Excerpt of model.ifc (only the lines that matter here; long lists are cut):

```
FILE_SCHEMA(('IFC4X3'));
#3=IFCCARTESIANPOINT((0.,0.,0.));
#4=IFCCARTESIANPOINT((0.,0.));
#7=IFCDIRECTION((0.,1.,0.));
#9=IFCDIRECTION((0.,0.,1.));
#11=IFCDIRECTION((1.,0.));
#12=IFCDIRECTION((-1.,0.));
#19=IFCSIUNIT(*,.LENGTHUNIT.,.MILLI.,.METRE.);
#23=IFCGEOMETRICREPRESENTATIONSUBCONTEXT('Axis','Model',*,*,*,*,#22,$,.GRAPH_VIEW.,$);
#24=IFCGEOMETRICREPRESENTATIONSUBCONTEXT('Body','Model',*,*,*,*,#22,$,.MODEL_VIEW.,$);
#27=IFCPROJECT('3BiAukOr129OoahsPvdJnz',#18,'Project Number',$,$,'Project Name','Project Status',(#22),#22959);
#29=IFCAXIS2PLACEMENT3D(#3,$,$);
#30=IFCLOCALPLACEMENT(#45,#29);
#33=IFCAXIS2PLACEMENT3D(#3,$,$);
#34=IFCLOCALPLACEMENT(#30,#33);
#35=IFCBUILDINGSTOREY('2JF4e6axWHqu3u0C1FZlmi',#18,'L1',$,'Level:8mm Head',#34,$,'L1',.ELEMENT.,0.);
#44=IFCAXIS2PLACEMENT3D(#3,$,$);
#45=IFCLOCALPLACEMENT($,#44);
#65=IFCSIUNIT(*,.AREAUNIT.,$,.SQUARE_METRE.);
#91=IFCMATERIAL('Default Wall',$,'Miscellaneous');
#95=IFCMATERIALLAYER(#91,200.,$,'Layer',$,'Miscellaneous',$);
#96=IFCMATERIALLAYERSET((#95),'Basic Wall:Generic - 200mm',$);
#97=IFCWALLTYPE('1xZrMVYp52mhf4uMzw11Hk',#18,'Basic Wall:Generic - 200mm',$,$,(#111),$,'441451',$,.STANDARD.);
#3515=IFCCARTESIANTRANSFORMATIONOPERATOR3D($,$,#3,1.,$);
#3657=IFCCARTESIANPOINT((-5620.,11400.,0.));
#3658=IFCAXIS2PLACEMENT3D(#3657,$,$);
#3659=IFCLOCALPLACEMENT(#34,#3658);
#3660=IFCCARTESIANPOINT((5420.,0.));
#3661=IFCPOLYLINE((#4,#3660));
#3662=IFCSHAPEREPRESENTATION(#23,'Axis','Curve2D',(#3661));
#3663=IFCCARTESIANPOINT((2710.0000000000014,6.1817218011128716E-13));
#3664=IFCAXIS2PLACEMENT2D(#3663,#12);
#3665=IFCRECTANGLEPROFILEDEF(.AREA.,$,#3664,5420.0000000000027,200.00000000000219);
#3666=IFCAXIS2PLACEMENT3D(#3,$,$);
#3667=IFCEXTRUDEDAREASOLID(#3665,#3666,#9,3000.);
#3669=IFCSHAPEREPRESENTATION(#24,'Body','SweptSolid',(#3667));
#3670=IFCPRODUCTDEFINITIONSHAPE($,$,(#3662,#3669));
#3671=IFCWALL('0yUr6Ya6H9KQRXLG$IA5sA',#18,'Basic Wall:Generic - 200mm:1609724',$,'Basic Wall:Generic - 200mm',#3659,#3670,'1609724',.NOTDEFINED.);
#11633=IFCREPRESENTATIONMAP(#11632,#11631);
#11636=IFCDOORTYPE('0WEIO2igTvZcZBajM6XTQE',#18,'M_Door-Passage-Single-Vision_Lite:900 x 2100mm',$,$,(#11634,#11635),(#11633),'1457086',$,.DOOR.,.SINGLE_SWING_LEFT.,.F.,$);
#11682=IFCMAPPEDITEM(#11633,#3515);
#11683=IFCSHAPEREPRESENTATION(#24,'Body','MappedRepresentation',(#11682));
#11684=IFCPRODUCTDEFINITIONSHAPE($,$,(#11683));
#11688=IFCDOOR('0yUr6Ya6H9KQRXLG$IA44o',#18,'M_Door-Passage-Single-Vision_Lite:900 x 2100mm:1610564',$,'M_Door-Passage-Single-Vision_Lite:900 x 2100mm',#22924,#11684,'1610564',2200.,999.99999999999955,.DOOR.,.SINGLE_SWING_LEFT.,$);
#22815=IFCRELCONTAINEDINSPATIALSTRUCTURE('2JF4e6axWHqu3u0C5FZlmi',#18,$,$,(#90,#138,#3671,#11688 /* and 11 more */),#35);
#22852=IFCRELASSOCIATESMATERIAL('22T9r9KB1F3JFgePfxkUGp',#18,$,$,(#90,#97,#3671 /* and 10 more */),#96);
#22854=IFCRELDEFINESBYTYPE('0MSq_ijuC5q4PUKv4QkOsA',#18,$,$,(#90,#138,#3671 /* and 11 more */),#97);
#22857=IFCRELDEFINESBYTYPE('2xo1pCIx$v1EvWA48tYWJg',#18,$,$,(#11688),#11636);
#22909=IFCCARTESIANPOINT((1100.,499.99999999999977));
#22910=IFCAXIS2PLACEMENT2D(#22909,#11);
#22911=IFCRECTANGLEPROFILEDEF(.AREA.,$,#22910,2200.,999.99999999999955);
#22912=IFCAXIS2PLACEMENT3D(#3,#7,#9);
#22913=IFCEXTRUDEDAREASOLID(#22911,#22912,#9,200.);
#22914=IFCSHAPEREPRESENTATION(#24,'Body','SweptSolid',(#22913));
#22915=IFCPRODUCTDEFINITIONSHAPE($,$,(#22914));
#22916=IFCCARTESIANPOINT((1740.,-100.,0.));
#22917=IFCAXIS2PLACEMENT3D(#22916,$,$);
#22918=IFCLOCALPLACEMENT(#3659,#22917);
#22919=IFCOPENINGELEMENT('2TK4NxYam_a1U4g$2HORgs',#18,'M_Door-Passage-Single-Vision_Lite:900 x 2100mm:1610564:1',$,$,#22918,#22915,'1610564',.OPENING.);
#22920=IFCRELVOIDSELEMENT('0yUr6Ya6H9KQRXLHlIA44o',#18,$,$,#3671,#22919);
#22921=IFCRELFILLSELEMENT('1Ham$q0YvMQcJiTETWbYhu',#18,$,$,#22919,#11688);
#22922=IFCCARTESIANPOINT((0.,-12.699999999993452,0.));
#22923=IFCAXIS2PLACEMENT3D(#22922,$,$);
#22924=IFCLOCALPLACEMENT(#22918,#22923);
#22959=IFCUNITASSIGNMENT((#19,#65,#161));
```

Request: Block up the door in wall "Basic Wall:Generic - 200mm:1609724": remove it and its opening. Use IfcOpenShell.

```python
import ifcopenshell
import ifcopenshell.api.feature
import ifcopenshell.api.root
import ifcopenshell.geom
import ifcopenshell.util.shape

model = ifcopenshell.open("model.ifc")
settings = ifcopenshell.geom.settings()


def volume(element):
    """Net volume in cubic metres, openings subtracted."""
    shape = ifcopenshell.geom.create_shape(settings, element)
    return ifcopenshell.util.shape.get_volume(shape.geometry)


door = model.by_guid("0yUr6Ya6H9KQRXLG$IA44o")
opening = door.FillsVoids[0].RelatingOpeningElement
wall = opening.VoidsElements[0].RelatingBuildingElement
before = volume(wall)

ifcopenshell.api.root.remove_product(model, product=door)
ifcopenshell.api.feature.remove_feature(model, feature=opening)

after = volume(wall)

print(f"wall volume {before:.3f} -> {after:.3f} m3")

model.write("model-out.ifc")
```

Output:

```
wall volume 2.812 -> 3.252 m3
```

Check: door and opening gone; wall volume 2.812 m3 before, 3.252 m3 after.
